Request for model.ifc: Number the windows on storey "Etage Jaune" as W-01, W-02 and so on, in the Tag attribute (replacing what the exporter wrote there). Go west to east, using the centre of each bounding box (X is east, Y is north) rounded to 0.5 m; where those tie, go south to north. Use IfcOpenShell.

First a look at what the model holds.

```python
import ifcopenshell
import ifcopenshell.util.element
import ifcopenshell.util.placement

model = ifcopenshell.open("model.ifc")
print(model.schema)
storey = next(s for s in model.by_type("IfcBuildingStorey") if s.Name == "Etage Jaune")
windows = [e for e in ifcopenshell.util.element.get_decomposition(storey) if e.is_a("IfcWindow")]
for e in sorted(windows, key=lambda e: e.id()):
    origin = ifcopenshell.util.placement.get_local_placement(e.ObjectPlacement)[:3, 3]
    print(e.id(), e.Tag, e.Name, origin.round(2) + 0.0, sep=" | ")
```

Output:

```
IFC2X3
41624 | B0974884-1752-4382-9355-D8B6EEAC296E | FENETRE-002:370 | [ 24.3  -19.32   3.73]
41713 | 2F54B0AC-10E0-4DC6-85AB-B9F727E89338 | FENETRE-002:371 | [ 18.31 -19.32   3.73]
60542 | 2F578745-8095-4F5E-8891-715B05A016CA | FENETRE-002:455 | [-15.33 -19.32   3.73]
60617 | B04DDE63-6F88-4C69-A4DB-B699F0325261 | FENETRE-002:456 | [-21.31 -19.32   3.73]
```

```python
import ifcopenshell
import ifcopenshell.geom
import ifcopenshell.util.element
import ifcopenshell.util.shape

model = ifcopenshell.open("model.ifc")
settings = ifcopenshell.geom.settings()
settings.set("use-world-coords", True)


def centre(element):
    shape = ifcopenshell.geom.create_shape(settings, element)
    return ifcopenshell.util.shape.get_bbox_centroid(shape.geometry)


storey = next(s for s in model.by_type("IfcBuildingStorey") if s.Name == "Etage Jaune")
windows = [e for e in ifcopenshell.util.element.get_decomposition(storey) if e.is_a("IfcWindow")]

# Insertion points can sit at a corner or the storey origin, so sort by the geometry (in metres).
centres = {e: centre(e) for e in windows}
windows.sort(key=lambda e: (round(centres[e][0] / 0.5), centres[e][1]))

for i, e in enumerate(windows, start=1):
    number = f"W-{i:02d}"
    e.Tag = number
    print(e.id(), number)

model.write("model-out.ifc")
```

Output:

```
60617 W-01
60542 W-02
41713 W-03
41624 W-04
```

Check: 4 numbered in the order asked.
